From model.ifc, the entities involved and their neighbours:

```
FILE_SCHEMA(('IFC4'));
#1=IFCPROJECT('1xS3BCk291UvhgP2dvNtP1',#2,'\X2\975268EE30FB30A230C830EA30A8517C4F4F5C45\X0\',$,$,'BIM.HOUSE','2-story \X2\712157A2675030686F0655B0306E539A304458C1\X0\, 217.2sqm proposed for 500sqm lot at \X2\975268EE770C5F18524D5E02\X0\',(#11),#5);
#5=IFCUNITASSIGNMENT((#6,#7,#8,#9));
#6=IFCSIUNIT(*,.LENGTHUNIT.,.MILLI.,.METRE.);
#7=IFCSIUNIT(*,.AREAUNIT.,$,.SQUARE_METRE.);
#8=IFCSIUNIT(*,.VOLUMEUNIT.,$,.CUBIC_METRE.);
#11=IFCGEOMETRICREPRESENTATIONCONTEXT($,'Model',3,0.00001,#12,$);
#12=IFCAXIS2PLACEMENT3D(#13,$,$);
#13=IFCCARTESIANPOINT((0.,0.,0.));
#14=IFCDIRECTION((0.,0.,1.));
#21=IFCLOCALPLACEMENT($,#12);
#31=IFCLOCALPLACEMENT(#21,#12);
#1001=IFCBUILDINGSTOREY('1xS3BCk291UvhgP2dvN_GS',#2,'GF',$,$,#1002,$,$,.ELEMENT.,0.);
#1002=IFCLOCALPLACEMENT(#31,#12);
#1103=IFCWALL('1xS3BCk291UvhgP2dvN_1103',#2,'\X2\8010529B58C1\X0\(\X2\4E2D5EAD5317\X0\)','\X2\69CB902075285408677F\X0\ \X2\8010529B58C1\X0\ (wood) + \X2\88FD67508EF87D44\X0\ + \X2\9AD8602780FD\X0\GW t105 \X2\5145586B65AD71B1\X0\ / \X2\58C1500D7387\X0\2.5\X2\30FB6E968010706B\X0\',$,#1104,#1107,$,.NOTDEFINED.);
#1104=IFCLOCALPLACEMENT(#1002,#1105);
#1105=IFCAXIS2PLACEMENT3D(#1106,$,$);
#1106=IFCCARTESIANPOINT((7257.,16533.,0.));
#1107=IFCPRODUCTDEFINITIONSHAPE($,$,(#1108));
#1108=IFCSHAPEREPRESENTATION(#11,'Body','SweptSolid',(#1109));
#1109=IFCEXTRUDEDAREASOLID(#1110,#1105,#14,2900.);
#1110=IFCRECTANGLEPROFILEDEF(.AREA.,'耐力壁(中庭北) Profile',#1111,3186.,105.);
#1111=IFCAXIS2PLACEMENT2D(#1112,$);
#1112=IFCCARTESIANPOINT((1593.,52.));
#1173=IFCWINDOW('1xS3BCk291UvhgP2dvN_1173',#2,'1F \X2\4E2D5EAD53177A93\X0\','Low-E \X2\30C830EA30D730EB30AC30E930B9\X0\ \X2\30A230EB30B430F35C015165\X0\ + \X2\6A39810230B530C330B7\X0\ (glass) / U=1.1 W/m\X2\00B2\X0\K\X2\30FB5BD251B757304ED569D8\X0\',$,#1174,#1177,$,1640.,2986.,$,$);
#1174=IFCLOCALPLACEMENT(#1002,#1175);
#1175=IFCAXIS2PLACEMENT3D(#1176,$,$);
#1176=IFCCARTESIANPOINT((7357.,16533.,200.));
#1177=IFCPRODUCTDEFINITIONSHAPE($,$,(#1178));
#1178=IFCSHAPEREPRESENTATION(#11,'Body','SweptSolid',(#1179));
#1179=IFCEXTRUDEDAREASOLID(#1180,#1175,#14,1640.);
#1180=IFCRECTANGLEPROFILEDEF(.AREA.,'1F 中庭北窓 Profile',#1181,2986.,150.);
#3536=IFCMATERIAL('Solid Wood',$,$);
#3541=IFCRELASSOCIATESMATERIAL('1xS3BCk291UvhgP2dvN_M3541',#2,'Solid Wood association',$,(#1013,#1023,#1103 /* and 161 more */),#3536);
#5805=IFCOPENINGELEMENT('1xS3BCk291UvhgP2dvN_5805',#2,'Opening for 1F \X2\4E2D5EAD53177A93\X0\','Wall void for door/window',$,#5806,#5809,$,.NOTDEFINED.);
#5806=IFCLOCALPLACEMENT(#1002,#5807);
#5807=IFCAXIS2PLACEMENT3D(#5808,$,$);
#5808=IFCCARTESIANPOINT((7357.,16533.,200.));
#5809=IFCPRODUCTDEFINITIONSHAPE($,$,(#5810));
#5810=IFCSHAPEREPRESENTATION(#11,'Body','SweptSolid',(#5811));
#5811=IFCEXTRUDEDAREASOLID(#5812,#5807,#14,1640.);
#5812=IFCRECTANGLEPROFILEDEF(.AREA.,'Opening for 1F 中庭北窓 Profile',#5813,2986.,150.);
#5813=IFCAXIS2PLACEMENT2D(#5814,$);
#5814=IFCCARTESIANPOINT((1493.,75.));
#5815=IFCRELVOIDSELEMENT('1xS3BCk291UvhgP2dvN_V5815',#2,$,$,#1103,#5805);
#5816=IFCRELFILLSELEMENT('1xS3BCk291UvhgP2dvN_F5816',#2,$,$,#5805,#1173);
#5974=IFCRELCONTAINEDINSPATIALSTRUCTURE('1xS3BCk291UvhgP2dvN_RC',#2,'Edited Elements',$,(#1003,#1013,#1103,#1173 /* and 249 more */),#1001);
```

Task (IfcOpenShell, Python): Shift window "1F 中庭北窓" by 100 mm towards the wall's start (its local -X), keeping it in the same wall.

```python
import ifcopenshell
import ifcopenshell.api.geometry
import ifcopenshell.util.placement
import ifcopenshell.util.unit

model = ifcopenshell.open("model.ifc")
unit_scale = ifcopenshell.util.unit.calculate_unit_scale(model)

window = model.by_guid("1xS3BCk291UvhgP2dvN_1173")
opening = window.FillsVoids[0].RelatingOpeningElement
wall = opening.VoidsElements[0].RelatingBuildingElement

wall_matrix = ifcopenshell.util.placement.get_local_placement(wall.ObjectPlacement)
shift = wall_matrix[:3, 0] * -0.1 / unit_scale
before = ifcopenshell.util.placement.get_local_placement(window.ObjectPlacement)[:3, 3].copy()

# The window is not placed relative to its opening, so move both.
for product in (opening, window):
    matrix = ifcopenshell.util.placement.get_local_placement(product.ObjectPlacement)
    matrix[:3, 3] += shift
    ifcopenshell.api.geometry.edit_object_placement(model, product=product, matrix=matrix, is_si=False)

after = ifcopenshell.util.placement.get_local_placement(window.ObjectPlacement)[:3, 3]
print("window moved by", (after - before).round(3) + 0.0)

model.write("model_edited.ifc")
```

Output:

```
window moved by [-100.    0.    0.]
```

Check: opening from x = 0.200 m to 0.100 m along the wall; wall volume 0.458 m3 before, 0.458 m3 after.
